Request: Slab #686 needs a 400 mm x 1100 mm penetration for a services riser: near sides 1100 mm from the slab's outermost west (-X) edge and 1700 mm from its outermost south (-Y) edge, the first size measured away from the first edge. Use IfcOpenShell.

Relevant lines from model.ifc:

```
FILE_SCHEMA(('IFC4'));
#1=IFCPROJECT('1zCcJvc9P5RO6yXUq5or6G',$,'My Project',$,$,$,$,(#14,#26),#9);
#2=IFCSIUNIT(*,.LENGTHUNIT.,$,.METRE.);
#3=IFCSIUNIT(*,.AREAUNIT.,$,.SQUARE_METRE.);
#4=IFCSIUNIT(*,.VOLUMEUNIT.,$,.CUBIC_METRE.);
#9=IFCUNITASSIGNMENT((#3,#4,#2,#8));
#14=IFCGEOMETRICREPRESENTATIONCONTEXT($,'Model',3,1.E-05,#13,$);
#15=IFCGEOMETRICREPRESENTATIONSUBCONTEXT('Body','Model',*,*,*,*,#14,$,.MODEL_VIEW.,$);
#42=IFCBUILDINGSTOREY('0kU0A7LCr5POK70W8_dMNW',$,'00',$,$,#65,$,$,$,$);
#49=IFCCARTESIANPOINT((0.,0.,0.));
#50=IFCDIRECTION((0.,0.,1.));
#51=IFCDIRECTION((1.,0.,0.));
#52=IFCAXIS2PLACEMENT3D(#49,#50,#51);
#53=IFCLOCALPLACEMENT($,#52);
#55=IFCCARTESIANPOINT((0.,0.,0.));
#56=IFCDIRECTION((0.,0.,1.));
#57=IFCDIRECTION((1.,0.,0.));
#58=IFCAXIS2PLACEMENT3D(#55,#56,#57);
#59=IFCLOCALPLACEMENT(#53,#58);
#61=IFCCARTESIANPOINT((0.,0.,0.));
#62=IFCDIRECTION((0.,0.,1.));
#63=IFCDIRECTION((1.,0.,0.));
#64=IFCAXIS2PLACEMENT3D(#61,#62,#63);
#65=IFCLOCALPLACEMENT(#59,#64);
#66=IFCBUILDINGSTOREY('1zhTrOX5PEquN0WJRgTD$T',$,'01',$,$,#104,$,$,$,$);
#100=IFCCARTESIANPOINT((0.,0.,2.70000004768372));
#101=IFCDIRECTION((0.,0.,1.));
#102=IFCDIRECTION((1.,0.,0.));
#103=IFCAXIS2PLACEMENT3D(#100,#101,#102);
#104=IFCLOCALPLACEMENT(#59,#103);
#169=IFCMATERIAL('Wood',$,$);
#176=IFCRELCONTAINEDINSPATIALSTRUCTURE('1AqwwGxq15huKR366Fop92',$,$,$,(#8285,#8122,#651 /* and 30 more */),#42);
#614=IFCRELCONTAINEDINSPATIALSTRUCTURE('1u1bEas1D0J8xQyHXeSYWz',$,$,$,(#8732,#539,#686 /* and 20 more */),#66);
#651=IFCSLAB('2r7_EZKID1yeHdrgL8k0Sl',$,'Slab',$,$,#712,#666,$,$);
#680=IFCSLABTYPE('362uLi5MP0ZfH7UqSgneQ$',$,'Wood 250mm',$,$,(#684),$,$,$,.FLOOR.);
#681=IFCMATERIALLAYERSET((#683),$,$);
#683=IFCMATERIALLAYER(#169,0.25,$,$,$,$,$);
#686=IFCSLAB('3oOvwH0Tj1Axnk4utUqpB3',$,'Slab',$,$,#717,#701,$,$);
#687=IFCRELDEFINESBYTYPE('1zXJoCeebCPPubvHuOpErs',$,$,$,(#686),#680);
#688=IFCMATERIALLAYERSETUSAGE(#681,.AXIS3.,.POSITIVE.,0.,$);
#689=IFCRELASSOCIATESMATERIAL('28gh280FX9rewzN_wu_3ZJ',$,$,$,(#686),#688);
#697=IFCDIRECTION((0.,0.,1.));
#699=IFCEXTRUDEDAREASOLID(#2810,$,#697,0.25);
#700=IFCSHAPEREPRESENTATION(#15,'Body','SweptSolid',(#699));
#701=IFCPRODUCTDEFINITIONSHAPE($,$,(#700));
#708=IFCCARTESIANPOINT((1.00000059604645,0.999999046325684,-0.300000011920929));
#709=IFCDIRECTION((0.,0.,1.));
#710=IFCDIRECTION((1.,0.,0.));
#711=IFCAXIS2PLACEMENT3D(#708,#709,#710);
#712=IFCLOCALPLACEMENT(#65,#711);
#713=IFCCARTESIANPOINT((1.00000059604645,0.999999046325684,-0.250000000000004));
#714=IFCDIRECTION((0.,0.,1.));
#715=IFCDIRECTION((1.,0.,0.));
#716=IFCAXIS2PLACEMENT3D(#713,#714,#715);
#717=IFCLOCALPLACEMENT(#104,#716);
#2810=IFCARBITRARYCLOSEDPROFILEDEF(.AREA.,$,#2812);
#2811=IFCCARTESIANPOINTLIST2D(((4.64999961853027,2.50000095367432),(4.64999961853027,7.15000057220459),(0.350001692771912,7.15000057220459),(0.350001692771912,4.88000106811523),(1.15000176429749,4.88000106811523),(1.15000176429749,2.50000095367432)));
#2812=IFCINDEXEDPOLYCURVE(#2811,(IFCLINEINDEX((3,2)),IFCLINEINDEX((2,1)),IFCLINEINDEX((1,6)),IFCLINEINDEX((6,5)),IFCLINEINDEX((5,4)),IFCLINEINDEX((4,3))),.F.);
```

```python
import numpy as np
import ifcopenshell
import ifcopenshell.api.feature
import ifcopenshell.api.geometry
import ifcopenshell.api.root
import ifcopenshell.geom
import ifcopenshell.util.placement
import ifcopenshell.util.representation
import ifcopenshell.util.shape
import ifcopenshell.util.unit

model = ifcopenshell.open("model.ifc")
unit_scale = ifcopenshell.util.unit.calculate_unit_scale(model)
settings = ifcopenshell.geom.settings()


def volume(element):
    """Net volume in cubic metres, openings subtracted."""
    shape = ifcopenshell.geom.create_shape(settings, element)
    return ifcopenshell.util.shape.get_volume(shape.geometry)


slab = model.by_id(686)
before = volume(slab)

# Extent in the slab's own axes, in metres. The edges named are its -X and -Y sides.
slab_shape = ifcopenshell.geom.create_shape(settings, slab)
vertices = ifcopenshell.util.shape.get_vertices(slab_shape.geometry)
x_min, y_min, bottom = vertices.min(axis=0)
top = vertices[:, 2].max()

opening = ifcopenshell.api.root.create_entity(model, ifc_class="IfcOpeningElement", name="Services riser opening", predefined_type="OPENING")
context = ifcopenshell.util.representation.get_context(model, "Model", "Body", "MODEL_VIEW")
width, depth = 0.4, 1.1
outline = [(0.0, 0.0), (width, 0.0), (width, depth), (0.0, depth), (0.0, 0.0)]
# Overshoot both faces by 50 mm so the cut is clean.
shape = ifcopenshell.api.geometry.add_slab_representation(
    model, context=context, depth=top - bottom + 0.1, polyline=outline
)
ifcopenshell.api.geometry.assign_representation(model, product=opening, representation=shape)

matrix = ifcopenshell.util.placement.get_local_placement(slab.ObjectPlacement)
matrix[:, 3] = matrix @ np.append(np.array([x_min + 1.1, y_min + 1.7, bottom - 0.05]) / unit_scale, 1.0)
ifcopenshell.api.geometry.edit_object_placement(model, product=opening, matrix=matrix, is_si=False)
ifcopenshell.api.feature.add_feature(model, feature=opening, element=slab)

after = volume(slab)

print(f"slab volume {before:.3f} -> {after:.3f} m3")

model.write("model_rev.ifc")
```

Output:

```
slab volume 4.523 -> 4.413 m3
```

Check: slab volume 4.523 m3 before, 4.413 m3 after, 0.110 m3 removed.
